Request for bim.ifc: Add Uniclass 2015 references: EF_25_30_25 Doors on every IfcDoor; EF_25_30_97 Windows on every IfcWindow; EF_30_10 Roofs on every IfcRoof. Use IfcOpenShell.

First a look at what the model holds.

```python
import ifcopenshell

model = ifcopenshell.open("bim.ifc")
print(model.schema)
print("classifications:", [c.Name for c in model.by_type("IfcClassification")])
for ifc_class in ("IfcDoor", "IfcRoof", "IfcStair", "IfcWall", "IfcWindow"):
    print(ifc_class, len(model.by_type(ifc_class)))
```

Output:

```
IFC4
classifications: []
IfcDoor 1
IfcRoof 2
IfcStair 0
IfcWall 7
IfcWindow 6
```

```python
import ifcopenshell
import ifcopenshell.api.classification

model = ifcopenshell.open("bim.ifc")

system = ifcopenshell.api.classification.add_classification(model, classification="Uniclass 2015")

codes = {
    "IfcDoor": ("EF_25_30_25", "Doors"),
    "IfcWindow": ("EF_25_30_97", "Windows"),
    "IfcRoof": ("EF_30_10", "Roofs"),
}
for ifc_class, (code, name) in codes.items():
    products = model.by_type(ifc_class)
    ifcopenshell.api.classification.add_reference(
        model, products=products, classification=system, identification=code, name=name
    )
    print(code, len(products))

model.write("bim_edited.ifc")
```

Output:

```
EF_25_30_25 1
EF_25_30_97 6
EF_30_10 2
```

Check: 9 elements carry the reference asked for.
